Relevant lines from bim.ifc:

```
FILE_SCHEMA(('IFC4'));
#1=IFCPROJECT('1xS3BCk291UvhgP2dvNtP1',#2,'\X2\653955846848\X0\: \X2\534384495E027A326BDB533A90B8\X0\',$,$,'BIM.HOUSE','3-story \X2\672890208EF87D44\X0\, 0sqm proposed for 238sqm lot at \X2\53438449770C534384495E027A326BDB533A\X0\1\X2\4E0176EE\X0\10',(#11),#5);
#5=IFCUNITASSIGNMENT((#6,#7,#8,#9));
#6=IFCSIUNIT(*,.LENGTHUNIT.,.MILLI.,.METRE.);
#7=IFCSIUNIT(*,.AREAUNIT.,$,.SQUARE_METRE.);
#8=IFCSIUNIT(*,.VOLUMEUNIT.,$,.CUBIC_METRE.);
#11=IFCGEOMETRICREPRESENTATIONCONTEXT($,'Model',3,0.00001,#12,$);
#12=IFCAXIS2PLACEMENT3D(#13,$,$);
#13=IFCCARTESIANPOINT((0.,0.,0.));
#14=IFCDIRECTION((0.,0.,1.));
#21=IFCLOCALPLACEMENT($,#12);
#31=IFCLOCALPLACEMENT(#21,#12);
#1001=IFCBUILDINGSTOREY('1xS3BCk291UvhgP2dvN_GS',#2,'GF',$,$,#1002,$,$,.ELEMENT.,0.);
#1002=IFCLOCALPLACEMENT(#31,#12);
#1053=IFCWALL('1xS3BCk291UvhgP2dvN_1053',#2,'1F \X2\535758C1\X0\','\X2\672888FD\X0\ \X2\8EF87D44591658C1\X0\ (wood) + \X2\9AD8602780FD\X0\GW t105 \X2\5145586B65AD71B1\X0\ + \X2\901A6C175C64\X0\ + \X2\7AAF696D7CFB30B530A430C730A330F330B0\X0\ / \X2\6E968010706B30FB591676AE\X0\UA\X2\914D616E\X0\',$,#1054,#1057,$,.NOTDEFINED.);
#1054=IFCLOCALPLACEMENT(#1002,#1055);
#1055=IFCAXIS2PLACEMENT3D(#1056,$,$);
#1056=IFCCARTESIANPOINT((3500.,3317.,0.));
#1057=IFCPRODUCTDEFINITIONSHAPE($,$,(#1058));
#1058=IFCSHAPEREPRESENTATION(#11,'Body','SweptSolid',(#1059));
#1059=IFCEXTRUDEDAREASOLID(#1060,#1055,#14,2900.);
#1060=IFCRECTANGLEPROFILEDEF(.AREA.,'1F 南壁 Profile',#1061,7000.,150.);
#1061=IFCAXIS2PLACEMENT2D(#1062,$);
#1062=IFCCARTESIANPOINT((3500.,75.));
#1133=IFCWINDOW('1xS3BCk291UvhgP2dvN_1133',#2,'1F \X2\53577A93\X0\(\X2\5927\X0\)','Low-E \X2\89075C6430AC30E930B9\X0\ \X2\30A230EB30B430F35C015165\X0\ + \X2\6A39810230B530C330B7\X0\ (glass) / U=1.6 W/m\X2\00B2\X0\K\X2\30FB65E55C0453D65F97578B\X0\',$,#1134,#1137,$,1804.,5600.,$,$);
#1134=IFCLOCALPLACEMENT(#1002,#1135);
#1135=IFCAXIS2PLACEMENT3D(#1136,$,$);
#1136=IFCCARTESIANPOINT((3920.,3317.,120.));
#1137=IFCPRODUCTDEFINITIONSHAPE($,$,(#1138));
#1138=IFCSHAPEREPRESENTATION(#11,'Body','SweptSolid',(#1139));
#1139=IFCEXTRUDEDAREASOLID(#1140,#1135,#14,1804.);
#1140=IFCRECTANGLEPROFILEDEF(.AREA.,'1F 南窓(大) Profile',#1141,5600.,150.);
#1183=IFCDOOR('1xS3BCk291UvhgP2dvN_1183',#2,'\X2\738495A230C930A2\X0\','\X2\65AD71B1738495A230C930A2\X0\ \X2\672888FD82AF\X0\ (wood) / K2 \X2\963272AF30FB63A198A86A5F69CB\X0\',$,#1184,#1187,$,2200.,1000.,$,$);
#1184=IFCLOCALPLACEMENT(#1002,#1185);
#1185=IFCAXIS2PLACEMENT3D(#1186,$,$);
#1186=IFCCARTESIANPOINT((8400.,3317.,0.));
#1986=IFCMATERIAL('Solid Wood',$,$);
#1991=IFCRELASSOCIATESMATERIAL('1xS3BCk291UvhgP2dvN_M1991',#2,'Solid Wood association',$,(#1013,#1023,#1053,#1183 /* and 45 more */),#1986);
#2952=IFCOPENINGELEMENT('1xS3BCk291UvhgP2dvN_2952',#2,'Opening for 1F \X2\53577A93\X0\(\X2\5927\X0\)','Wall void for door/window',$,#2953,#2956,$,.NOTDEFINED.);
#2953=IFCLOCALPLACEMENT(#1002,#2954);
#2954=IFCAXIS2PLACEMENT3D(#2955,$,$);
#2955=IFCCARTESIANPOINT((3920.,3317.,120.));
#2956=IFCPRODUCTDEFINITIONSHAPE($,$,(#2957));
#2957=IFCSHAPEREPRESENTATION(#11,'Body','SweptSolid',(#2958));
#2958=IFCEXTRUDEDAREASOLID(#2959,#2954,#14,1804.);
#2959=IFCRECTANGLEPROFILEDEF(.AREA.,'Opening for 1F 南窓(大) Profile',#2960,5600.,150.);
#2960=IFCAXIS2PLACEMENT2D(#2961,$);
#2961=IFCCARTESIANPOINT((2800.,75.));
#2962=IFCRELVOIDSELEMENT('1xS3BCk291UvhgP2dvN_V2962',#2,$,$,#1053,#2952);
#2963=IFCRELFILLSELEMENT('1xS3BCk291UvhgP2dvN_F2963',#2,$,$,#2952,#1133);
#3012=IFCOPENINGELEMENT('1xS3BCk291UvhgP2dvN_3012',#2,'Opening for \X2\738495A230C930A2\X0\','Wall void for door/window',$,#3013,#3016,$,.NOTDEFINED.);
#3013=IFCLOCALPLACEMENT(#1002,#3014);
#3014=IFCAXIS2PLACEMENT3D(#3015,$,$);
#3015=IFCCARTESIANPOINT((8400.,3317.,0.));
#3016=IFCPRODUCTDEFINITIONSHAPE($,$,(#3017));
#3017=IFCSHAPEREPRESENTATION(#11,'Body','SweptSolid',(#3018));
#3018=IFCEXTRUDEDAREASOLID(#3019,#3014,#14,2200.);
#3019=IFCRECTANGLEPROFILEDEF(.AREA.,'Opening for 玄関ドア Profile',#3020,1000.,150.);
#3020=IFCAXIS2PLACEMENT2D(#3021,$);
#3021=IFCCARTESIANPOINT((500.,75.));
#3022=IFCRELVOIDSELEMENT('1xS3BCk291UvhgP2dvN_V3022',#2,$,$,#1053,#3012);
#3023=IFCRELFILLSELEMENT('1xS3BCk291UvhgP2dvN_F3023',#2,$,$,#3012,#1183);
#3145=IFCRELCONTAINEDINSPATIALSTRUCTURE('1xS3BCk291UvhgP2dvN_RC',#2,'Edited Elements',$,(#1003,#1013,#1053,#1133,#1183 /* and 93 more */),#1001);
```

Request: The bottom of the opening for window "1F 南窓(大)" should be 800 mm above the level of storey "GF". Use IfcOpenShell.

```python
import numpy as np
import ifcopenshell
import ifcopenshell.api.geometry
import ifcopenshell.geom
import ifcopenshell.util.element
import ifcopenshell.util.placement
import ifcopenshell.util.shape
import ifcopenshell.util.unit

model = ifcopenshell.open("bim.ifc")
unit_scale = ifcopenshell.util.unit.calculate_unit_scale(model)

window = model.by_guid("1xS3BCk291UvhgP2dvN_1133")
opening = window.FillsVoids[0].RelatingOpeningElement
storey = ifcopenshell.util.element.get_container(window, ifc_class="IfcBuildingStorey")
level = ifcopenshell.util.placement.get_local_placement(storey.ObjectPlacement)[2, 3]

# The opening's origin need not be at the sill, so measure its lowest point.
shape = ifcopenshell.geom.create_shape(ifcopenshell.geom.settings(), opening)
bottom = ifcopenshell.util.shape.get_shape_bottom_elevation(shape, shape.geometry) / unit_scale
dz = level + 800.0 - bottom

shift = np.array([0.0, 0.0, dz])
# The window is not placed relative to its opening, so move both.
for product in (opening, window):
    matrix = ifcopenshell.util.placement.get_local_placement(product.ObjectPlacement)
    matrix[:3, 3] += shift
    ifcopenshell.api.geometry.edit_object_placement(model, product=product, matrix=matrix, is_si=False)

print(f"moved by {dz * unit_scale:+.3f} m")

model.write("bim_v2.ifc")
```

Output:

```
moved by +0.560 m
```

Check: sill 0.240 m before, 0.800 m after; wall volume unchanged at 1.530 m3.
